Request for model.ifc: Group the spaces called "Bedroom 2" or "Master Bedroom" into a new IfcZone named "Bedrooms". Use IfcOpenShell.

First a look at what the model holds.

```python
import ifcopenshell

model = ifcopenshell.open("model.ifc")
print(model.schema)
seen = {}
for space in model.by_type("IfcSpace"):
    seen[space.LongName] = seen.get(space.LongName, 0) + 1
for name, count in sorted(seen.items(), key=str):
    print(count, "x", name)
print("zones:", [z.Name for z in model.by_type("IfcZone")][:20])
```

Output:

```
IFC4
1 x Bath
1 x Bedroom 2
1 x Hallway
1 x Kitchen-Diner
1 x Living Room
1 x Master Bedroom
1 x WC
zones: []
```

```python
import ifcopenshell
import ifcopenshell.api.group
import ifcopenshell.api.root

model = ifcopenshell.open("model.ifc")

names = {"Bedroom 2", "Master Bedroom"}
spaces = [s for s in model.by_type("IfcSpace") if s.LongName in names]

zone = ifcopenshell.api.root.create_entity(model, ifc_class="IfcZone", name="Bedrooms")
ifcopenshell.api.group.assign_group(model, products=spaces, group=zone)
print(len(spaces), "spaces in", zone.Name)

model.write("model_v2.ifc")
```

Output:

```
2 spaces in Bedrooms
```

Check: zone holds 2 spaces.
